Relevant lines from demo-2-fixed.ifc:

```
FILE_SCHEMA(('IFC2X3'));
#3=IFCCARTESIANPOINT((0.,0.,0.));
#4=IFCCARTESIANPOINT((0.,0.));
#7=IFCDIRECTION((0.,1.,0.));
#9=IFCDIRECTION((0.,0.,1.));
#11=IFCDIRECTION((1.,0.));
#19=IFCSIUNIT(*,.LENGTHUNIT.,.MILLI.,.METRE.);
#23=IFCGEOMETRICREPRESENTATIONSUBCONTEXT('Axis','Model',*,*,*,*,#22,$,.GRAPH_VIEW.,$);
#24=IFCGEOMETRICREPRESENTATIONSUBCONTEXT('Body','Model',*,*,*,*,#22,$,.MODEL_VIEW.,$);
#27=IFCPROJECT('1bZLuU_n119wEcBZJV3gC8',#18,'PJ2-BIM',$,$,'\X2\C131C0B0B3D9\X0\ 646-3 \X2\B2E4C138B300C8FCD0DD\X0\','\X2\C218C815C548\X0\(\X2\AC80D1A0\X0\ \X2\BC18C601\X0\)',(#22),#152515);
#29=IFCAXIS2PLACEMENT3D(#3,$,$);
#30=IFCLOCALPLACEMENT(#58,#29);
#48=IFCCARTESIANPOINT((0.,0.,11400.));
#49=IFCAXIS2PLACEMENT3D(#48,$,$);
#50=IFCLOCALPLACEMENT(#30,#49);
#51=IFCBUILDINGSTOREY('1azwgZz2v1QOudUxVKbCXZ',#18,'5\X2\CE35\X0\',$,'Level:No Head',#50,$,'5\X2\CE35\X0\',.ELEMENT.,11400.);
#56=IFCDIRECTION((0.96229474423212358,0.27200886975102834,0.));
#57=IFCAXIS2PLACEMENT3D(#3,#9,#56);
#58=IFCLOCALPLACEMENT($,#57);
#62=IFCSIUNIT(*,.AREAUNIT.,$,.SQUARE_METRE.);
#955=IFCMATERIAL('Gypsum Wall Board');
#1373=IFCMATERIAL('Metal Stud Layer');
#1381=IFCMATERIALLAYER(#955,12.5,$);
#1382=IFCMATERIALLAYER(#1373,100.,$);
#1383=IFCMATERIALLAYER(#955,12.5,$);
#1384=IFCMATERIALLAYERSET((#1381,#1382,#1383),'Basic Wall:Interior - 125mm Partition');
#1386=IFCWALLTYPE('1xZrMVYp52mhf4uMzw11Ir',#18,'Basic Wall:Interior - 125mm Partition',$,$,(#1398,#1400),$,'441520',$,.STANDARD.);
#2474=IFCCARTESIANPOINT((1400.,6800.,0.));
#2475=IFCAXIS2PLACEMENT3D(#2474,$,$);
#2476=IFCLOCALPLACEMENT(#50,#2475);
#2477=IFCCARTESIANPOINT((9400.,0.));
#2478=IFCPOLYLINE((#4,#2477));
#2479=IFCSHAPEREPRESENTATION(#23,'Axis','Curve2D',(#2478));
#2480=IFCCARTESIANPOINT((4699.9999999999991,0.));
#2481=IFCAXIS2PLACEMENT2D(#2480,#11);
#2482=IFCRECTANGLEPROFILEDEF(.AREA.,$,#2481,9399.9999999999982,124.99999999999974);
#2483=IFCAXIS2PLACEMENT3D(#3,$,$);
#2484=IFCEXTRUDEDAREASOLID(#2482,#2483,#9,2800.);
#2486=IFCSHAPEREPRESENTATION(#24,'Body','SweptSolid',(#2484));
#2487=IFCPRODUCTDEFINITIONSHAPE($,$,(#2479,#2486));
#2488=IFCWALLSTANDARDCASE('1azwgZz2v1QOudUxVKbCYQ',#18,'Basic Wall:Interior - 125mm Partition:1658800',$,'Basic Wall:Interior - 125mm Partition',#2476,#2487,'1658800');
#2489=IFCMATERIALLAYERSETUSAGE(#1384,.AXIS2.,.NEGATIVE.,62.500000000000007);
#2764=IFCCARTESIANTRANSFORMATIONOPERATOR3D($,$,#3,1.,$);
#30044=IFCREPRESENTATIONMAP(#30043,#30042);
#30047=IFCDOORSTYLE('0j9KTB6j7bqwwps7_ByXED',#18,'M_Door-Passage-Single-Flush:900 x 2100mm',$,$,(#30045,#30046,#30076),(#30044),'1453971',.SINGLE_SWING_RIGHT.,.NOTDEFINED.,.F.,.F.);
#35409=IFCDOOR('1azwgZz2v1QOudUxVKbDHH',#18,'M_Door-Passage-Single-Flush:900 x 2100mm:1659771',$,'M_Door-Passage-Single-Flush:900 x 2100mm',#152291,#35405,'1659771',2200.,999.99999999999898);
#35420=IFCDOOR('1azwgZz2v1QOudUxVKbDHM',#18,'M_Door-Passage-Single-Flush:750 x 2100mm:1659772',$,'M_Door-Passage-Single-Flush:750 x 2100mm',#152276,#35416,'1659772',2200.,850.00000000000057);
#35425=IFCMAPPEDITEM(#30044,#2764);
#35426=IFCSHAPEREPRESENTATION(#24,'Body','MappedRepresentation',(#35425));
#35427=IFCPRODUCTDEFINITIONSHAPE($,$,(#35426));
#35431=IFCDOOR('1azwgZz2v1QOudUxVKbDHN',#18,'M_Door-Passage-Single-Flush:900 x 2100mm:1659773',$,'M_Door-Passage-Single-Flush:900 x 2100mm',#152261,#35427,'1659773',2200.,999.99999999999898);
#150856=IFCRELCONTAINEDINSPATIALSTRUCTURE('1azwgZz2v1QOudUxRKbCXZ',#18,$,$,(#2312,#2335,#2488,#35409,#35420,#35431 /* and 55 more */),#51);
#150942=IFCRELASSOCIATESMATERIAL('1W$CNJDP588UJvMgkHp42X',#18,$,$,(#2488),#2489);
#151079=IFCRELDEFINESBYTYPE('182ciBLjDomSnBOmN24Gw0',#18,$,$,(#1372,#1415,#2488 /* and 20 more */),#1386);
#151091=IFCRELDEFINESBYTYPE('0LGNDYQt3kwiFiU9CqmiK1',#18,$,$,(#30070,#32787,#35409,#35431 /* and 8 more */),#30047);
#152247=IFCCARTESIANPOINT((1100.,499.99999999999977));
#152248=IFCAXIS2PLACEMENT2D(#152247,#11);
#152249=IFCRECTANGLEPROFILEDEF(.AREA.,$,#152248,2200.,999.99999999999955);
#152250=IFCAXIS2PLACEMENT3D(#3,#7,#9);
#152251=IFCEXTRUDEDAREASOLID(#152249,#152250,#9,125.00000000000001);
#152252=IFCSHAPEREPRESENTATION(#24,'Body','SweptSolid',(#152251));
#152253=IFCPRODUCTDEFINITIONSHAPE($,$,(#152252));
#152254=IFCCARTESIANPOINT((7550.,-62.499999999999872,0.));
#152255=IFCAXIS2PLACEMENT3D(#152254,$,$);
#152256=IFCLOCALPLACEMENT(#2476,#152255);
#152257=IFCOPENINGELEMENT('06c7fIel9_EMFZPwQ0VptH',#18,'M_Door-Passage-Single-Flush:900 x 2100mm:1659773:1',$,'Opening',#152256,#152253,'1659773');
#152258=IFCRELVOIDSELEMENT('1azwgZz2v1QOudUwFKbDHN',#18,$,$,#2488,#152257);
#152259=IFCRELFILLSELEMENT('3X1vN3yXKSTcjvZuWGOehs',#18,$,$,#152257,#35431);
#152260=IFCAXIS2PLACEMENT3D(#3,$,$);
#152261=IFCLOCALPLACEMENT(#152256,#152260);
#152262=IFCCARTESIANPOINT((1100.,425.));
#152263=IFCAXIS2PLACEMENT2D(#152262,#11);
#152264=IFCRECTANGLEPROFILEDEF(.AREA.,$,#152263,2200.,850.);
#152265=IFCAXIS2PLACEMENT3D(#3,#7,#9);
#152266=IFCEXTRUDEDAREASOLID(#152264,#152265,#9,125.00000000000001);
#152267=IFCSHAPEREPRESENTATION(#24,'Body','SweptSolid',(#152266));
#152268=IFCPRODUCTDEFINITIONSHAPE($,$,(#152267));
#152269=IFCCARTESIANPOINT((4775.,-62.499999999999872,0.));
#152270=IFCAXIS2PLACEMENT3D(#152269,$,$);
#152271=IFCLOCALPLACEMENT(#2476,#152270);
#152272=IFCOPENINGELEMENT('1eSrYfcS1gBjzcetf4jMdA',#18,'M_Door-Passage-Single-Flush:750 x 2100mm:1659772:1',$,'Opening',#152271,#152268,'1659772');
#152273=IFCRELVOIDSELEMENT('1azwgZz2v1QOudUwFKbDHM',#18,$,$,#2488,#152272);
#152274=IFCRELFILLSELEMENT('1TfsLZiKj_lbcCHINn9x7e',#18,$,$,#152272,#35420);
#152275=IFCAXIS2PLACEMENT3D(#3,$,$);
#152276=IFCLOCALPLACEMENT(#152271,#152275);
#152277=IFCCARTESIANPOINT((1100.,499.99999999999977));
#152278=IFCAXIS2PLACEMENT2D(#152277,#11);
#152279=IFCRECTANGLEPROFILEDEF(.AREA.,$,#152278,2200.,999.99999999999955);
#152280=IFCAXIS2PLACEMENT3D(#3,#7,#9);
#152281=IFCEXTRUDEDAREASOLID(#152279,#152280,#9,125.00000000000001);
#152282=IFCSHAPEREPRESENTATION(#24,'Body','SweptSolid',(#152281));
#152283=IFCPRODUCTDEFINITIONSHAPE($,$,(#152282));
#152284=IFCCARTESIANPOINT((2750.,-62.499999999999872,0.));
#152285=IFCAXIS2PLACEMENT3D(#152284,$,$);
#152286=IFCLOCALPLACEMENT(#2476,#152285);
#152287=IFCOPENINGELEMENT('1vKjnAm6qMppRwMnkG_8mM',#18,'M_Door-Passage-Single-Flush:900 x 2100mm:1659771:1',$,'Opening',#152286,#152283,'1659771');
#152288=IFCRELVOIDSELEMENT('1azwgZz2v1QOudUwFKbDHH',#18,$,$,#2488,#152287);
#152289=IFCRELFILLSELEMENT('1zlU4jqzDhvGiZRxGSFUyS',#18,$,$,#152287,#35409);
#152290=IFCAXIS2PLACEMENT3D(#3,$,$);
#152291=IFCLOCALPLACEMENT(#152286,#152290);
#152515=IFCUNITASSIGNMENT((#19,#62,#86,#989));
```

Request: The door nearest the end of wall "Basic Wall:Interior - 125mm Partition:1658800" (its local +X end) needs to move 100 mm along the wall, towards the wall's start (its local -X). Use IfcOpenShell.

```python
import ifcopenshell
import ifcopenshell.api.geometry
import ifcopenshell.util.placement
import ifcopenshell.util.unit

model = ifcopenshell.open("demo-2-fixed.ifc")
unit_scale = ifcopenshell.util.unit.calculate_unit_scale(model)

door = model.by_guid("1azwgZz2v1QOudUxVKbDHN")
opening = door.FillsVoids[0].RelatingOpeningElement
wall = opening.VoidsElements[0].RelatingBuildingElement

wall_matrix = ifcopenshell.util.placement.get_local_placement(wall.ObjectPlacement)
shift = wall_matrix[:3, 0] * -0.1 / unit_scale
before = ifcopenshell.util.placement.get_local_placement(door.ObjectPlacement)[:3, 3].copy()

# The door is placed relative to its opening, so it follows when the opening moves.
matrix = ifcopenshell.util.placement.get_local_placement(opening.ObjectPlacement)
matrix[:3, 3] += shift
ifcopenshell.api.geometry.edit_object_placement(
    model, product=opening, matrix=matrix, is_si=False, should_transform_children=True
)

after = ifcopenshell.util.placement.get_local_placement(door.ObjectPlacement)[:3, 3]
print("door moved by", (after - before).round(3) + 0.0)

model.write("demo-2-fixed_edited.ifc")
```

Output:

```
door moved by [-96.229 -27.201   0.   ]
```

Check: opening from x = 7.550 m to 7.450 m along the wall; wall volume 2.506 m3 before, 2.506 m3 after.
